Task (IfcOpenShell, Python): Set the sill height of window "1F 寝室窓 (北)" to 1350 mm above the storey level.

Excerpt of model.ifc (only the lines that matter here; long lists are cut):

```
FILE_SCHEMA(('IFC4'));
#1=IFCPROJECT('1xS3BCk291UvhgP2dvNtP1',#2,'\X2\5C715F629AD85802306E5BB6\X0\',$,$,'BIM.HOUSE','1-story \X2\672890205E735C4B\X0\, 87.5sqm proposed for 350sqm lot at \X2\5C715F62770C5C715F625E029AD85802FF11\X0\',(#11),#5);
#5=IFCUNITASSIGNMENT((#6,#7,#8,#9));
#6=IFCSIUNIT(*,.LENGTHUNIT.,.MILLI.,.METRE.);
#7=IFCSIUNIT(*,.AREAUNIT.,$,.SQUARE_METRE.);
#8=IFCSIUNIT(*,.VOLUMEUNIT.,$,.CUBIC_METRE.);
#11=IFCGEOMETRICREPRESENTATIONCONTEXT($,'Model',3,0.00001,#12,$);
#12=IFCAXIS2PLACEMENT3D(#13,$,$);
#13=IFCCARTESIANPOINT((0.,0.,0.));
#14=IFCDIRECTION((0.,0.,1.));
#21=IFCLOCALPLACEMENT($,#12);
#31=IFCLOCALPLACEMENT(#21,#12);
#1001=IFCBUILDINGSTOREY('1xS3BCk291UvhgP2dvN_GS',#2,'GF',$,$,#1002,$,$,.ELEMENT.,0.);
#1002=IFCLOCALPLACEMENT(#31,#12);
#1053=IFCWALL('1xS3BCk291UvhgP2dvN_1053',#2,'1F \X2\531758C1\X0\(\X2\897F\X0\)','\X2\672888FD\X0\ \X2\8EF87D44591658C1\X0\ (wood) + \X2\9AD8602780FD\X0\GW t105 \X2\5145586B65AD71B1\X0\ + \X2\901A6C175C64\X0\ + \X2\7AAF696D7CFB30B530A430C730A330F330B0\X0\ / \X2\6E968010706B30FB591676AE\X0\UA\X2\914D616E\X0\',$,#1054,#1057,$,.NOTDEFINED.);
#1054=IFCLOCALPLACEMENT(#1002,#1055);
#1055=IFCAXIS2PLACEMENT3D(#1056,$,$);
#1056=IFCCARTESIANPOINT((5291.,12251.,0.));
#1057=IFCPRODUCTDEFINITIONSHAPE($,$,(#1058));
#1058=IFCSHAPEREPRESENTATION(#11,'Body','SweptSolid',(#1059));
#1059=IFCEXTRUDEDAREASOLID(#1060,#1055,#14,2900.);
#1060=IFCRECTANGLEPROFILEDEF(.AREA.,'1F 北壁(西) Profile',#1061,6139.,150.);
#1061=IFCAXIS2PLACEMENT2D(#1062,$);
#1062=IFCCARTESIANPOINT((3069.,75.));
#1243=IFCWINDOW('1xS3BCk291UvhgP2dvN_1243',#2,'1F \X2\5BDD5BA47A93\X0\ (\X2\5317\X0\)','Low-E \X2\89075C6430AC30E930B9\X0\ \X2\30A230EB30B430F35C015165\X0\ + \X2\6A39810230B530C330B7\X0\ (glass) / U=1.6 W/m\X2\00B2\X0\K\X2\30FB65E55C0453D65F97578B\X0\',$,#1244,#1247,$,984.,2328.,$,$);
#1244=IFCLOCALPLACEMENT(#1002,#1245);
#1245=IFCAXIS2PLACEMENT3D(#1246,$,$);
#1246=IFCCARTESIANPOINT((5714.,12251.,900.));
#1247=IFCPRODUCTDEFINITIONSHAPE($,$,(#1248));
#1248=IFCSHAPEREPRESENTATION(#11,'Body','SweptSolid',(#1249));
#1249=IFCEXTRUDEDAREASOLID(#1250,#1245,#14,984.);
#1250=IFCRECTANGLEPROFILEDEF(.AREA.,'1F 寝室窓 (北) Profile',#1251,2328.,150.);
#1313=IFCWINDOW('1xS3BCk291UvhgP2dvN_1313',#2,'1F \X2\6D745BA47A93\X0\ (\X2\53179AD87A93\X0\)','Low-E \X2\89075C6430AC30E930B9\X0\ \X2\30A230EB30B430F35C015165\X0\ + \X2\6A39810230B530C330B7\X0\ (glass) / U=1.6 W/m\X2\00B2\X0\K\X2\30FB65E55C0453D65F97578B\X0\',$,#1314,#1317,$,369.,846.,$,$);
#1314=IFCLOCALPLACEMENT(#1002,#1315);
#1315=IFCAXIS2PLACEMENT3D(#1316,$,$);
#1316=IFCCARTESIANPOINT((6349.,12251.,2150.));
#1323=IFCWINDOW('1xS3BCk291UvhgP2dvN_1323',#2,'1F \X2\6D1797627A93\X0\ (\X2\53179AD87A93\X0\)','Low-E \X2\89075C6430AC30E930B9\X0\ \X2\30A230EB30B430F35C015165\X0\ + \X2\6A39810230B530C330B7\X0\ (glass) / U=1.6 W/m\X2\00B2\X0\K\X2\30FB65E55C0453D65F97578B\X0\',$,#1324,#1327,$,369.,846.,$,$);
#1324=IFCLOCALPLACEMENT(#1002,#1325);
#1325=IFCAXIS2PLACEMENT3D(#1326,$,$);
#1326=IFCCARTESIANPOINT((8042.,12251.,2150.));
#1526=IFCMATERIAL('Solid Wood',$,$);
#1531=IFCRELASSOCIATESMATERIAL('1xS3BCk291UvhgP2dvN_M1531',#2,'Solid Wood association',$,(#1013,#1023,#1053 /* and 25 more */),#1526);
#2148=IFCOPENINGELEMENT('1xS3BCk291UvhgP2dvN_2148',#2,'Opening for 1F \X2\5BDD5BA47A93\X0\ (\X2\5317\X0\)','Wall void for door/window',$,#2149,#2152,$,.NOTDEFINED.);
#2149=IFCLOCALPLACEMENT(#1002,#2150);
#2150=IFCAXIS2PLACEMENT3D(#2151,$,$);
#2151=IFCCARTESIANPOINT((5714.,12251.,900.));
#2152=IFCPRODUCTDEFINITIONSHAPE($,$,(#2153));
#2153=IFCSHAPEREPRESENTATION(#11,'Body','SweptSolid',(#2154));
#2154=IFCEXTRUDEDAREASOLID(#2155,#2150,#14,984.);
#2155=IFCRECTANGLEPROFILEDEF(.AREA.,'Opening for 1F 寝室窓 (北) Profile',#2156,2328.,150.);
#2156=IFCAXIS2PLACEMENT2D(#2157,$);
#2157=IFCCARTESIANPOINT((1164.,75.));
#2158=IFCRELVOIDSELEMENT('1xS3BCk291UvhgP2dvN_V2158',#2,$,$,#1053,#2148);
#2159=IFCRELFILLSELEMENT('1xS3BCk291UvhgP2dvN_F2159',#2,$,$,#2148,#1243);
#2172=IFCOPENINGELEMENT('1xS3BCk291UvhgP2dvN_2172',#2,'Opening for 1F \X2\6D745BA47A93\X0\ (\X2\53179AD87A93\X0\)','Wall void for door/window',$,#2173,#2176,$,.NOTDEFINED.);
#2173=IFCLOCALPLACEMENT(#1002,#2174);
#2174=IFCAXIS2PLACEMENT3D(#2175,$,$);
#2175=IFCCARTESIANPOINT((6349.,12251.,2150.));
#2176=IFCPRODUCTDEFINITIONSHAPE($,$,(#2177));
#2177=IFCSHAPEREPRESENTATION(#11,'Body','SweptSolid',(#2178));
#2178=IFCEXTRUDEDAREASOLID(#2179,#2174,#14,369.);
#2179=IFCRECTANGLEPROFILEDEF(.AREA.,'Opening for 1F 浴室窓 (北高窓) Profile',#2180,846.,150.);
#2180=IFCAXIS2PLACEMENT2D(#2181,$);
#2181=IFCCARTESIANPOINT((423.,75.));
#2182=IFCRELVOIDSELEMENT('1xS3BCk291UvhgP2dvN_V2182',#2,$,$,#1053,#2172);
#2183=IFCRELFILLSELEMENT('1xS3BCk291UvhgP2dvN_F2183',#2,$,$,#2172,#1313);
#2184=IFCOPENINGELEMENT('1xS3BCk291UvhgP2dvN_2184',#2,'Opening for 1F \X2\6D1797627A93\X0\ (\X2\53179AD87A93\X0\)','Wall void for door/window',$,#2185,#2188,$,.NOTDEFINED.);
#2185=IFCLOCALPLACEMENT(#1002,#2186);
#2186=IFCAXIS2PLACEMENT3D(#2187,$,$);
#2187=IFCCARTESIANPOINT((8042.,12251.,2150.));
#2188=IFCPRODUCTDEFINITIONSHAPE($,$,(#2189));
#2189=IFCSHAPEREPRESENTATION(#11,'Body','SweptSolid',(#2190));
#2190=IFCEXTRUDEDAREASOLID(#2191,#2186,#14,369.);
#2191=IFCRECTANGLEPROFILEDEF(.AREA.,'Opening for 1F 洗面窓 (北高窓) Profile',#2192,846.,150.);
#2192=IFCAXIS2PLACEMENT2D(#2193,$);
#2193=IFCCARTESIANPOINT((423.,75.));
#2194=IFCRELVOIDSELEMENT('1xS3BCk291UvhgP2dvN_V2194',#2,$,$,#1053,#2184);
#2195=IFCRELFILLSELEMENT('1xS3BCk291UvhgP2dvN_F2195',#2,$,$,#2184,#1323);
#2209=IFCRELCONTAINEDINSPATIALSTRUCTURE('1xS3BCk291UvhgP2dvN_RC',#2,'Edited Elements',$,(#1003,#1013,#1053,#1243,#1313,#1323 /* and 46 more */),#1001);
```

```python
import numpy as np
import ifcopenshell
import ifcopenshell.api.geometry
import ifcopenshell.geom
import ifcopenshell.util.element
import ifcopenshell.util.placement
import ifcopenshell.util.shape
import ifcopenshell.util.unit

model = ifcopenshell.open("model.ifc")
unit_scale = ifcopenshell.util.unit.calculate_unit_scale(model)

window = model.by_guid("1xS3BCk291UvhgP2dvN_1243")
opening = window.FillsVoids[0].RelatingOpeningElement
storey = ifcopenshell.util.element.get_container(window, ifc_class="IfcBuildingStorey")
level = ifcopenshell.util.placement.get_local_placement(storey.ObjectPlacement)[2, 3]

# The opening's origin need not be at the sill, so measure its lowest point.
shape = ifcopenshell.geom.create_shape(ifcopenshell.geom.settings(), opening)
bottom = ifcopenshell.util.shape.get_shape_bottom_elevation(shape, shape.geometry) / unit_scale
dz = level + 1350.0 - bottom

shift = np.array([0.0, 0.0, dz])
# The window is not placed relative to its opening, so move both.
for product in (opening, window):
    matrix = ifcopenshell.util.placement.get_local_placement(product.ObjectPlacement)
    matrix[:3, 3] += shift
    ifcopenshell.api.geometry.edit_object_placement(model, product=product, matrix=matrix, is_si=False)

print(f"moved by {dz * unit_scale:+.3f} m")

model.write("model_edited.ifc")
```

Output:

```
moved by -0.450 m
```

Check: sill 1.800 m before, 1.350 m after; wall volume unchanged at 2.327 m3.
